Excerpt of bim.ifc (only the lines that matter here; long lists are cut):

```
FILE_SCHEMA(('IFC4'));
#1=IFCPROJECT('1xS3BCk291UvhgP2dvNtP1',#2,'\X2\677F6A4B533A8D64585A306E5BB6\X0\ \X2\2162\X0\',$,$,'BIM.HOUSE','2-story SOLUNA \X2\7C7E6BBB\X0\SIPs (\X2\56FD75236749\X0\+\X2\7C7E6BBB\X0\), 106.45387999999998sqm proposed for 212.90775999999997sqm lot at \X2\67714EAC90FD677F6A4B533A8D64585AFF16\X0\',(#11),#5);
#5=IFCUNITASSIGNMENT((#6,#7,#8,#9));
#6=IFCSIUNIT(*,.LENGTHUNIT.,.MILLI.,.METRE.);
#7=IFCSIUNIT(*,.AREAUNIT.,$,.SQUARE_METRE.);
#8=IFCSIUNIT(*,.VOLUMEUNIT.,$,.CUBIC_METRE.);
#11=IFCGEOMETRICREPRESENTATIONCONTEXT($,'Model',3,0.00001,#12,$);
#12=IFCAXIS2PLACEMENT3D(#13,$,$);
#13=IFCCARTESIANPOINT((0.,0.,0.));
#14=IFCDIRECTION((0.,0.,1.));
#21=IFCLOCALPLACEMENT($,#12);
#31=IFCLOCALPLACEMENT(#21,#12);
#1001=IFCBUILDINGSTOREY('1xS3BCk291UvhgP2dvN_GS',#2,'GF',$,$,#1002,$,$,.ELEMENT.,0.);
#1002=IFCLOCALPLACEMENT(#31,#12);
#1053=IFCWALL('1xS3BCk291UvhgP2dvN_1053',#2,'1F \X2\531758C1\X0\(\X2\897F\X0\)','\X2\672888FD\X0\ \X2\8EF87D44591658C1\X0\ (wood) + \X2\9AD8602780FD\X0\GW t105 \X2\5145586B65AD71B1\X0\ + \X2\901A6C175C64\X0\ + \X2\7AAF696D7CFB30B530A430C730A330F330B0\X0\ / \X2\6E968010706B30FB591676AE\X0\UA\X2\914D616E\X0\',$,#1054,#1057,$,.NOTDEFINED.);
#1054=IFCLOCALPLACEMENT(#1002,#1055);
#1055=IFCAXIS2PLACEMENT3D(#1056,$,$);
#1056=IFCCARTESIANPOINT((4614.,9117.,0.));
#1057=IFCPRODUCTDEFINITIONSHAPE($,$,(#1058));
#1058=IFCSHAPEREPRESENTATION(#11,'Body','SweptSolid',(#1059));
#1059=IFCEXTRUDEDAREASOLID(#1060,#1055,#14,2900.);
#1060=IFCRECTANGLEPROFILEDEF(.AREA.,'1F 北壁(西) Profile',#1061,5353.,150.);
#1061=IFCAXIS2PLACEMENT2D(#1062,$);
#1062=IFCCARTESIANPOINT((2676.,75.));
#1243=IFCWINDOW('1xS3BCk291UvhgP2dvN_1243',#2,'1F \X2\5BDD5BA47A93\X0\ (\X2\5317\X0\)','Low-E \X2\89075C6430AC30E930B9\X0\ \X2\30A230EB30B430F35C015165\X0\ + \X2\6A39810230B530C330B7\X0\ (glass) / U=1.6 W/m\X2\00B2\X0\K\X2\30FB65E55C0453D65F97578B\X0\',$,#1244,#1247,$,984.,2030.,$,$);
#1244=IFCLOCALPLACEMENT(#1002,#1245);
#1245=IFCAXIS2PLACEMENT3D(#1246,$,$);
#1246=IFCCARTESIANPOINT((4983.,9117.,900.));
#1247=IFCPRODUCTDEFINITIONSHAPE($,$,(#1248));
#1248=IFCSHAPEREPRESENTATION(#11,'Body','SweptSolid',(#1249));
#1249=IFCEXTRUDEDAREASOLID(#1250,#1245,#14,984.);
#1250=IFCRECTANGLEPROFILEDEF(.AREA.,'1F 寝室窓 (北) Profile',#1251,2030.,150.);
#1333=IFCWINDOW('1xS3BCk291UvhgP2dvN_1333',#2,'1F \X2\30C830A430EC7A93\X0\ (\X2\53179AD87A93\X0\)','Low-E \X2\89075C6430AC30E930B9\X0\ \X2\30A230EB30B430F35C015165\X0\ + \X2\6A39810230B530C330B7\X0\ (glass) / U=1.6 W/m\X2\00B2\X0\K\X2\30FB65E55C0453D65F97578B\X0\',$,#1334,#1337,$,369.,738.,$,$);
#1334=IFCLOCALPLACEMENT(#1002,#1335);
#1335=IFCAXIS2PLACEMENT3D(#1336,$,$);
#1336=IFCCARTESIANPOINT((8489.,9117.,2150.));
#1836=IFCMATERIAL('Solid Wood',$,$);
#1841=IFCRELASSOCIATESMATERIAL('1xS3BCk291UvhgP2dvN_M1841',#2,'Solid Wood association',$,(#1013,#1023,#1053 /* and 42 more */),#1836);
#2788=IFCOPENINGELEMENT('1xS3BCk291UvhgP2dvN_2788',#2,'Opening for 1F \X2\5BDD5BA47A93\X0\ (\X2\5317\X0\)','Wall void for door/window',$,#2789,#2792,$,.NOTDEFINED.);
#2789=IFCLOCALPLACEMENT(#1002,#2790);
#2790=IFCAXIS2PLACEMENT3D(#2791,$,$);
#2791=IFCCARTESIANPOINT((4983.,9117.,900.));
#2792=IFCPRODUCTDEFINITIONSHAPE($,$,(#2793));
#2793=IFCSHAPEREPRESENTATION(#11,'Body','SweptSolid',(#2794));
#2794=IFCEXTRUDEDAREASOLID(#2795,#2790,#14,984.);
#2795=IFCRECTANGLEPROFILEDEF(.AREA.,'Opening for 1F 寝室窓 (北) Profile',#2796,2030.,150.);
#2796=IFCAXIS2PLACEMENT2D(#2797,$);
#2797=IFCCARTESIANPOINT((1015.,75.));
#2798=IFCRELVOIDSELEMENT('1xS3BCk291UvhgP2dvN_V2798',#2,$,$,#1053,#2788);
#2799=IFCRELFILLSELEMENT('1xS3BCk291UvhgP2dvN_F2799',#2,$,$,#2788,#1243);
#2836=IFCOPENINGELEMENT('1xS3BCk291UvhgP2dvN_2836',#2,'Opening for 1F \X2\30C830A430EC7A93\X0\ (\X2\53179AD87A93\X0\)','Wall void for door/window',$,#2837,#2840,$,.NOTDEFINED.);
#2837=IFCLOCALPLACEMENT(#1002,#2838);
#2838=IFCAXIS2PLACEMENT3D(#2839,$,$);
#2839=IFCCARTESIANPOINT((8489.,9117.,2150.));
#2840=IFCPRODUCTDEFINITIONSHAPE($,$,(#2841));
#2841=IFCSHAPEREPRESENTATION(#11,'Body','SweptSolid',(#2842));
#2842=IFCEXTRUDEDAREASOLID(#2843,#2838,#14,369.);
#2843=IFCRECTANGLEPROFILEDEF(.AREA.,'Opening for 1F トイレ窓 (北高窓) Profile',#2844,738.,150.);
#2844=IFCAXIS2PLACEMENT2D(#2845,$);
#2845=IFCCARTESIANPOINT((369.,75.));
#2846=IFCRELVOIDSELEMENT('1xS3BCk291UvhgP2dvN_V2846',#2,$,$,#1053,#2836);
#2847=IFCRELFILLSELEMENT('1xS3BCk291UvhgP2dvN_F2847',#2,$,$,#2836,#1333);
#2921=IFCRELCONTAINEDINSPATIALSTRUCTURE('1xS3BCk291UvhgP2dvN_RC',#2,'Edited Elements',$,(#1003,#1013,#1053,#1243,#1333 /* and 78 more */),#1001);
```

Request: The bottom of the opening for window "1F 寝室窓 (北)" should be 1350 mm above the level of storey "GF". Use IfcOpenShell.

```python
import numpy as np
import ifcopenshell
import ifcopenshell.api.geometry
import ifcopenshell.geom
import ifcopenshell.util.element
import ifcopenshell.util.placement
import ifcopenshell.util.shape
import ifcopenshell.util.unit

model = ifcopenshell.open("bim.ifc")
unit_scale = ifcopenshell.util.unit.calculate_unit_scale(model)

window = model.by_guid("1xS3BCk291UvhgP2dvN_1243")
opening = window.FillsVoids[0].RelatingOpeningElement
storey = ifcopenshell.util.element.get_container(window, ifc_class="IfcBuildingStorey")
level = ifcopenshell.util.placement.get_local_placement(storey.ObjectPlacement)[2, 3]

# The opening's origin need not be at the sill, so measure its lowest point.
shape = ifcopenshell.geom.create_shape(ifcopenshell.geom.settings(), opening)
bottom = ifcopenshell.util.shape.get_shape_bottom_elevation(shape, shape.geometry) / unit_scale
dz = level + 1350.0 - bottom

shift = np.array([0.0, 0.0, dz])
# The window is not placed relative to its opening, so move both.
for product in (opening, window):
    matrix = ifcopenshell.util.placement.get_local_placement(product.ObjectPlacement)
    matrix[:3, 3] += shift
    ifcopenshell.api.geometry.edit_object_placement(model, product=product, matrix=matrix, is_si=False)

print(f"moved by {dz * unit_scale:+.3f} m")

model.write("bim_edited.ifc")
```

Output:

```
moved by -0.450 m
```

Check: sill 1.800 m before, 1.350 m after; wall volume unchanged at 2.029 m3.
